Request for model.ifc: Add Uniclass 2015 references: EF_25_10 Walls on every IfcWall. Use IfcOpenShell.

First a look at what the model holds.

```python
import ifcopenshell

model = ifcopenshell.open("model.ifc")
print(model.schema)
print("classifications:", [c.Name for c in model.by_type("IfcClassification")])
for ifc_class in ("IfcDoor", "IfcRoof", "IfcStair", "IfcWall", "IfcWindow"):
    print(ifc_class, len(model.by_type(ifc_class)))
```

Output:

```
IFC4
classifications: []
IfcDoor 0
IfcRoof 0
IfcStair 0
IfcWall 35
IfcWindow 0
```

```python
import ifcopenshell
import ifcopenshell.api.classification

model = ifcopenshell.open("model.ifc")

system = ifcopenshell.api.classification.add_classification(model, classification="Uniclass 2015")

codes = {
    "IfcWall": ("EF_25_10", "Walls"),
}
for ifc_class, (code, name) in codes.items():
    products = model.by_type(ifc_class)
    ifcopenshell.api.classification.add_reference(
        model, products=products, classification=system, identification=code, name=name
    )
    print(code, len(products))

model.write("model_updated.ifc")
```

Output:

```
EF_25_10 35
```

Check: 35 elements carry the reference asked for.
